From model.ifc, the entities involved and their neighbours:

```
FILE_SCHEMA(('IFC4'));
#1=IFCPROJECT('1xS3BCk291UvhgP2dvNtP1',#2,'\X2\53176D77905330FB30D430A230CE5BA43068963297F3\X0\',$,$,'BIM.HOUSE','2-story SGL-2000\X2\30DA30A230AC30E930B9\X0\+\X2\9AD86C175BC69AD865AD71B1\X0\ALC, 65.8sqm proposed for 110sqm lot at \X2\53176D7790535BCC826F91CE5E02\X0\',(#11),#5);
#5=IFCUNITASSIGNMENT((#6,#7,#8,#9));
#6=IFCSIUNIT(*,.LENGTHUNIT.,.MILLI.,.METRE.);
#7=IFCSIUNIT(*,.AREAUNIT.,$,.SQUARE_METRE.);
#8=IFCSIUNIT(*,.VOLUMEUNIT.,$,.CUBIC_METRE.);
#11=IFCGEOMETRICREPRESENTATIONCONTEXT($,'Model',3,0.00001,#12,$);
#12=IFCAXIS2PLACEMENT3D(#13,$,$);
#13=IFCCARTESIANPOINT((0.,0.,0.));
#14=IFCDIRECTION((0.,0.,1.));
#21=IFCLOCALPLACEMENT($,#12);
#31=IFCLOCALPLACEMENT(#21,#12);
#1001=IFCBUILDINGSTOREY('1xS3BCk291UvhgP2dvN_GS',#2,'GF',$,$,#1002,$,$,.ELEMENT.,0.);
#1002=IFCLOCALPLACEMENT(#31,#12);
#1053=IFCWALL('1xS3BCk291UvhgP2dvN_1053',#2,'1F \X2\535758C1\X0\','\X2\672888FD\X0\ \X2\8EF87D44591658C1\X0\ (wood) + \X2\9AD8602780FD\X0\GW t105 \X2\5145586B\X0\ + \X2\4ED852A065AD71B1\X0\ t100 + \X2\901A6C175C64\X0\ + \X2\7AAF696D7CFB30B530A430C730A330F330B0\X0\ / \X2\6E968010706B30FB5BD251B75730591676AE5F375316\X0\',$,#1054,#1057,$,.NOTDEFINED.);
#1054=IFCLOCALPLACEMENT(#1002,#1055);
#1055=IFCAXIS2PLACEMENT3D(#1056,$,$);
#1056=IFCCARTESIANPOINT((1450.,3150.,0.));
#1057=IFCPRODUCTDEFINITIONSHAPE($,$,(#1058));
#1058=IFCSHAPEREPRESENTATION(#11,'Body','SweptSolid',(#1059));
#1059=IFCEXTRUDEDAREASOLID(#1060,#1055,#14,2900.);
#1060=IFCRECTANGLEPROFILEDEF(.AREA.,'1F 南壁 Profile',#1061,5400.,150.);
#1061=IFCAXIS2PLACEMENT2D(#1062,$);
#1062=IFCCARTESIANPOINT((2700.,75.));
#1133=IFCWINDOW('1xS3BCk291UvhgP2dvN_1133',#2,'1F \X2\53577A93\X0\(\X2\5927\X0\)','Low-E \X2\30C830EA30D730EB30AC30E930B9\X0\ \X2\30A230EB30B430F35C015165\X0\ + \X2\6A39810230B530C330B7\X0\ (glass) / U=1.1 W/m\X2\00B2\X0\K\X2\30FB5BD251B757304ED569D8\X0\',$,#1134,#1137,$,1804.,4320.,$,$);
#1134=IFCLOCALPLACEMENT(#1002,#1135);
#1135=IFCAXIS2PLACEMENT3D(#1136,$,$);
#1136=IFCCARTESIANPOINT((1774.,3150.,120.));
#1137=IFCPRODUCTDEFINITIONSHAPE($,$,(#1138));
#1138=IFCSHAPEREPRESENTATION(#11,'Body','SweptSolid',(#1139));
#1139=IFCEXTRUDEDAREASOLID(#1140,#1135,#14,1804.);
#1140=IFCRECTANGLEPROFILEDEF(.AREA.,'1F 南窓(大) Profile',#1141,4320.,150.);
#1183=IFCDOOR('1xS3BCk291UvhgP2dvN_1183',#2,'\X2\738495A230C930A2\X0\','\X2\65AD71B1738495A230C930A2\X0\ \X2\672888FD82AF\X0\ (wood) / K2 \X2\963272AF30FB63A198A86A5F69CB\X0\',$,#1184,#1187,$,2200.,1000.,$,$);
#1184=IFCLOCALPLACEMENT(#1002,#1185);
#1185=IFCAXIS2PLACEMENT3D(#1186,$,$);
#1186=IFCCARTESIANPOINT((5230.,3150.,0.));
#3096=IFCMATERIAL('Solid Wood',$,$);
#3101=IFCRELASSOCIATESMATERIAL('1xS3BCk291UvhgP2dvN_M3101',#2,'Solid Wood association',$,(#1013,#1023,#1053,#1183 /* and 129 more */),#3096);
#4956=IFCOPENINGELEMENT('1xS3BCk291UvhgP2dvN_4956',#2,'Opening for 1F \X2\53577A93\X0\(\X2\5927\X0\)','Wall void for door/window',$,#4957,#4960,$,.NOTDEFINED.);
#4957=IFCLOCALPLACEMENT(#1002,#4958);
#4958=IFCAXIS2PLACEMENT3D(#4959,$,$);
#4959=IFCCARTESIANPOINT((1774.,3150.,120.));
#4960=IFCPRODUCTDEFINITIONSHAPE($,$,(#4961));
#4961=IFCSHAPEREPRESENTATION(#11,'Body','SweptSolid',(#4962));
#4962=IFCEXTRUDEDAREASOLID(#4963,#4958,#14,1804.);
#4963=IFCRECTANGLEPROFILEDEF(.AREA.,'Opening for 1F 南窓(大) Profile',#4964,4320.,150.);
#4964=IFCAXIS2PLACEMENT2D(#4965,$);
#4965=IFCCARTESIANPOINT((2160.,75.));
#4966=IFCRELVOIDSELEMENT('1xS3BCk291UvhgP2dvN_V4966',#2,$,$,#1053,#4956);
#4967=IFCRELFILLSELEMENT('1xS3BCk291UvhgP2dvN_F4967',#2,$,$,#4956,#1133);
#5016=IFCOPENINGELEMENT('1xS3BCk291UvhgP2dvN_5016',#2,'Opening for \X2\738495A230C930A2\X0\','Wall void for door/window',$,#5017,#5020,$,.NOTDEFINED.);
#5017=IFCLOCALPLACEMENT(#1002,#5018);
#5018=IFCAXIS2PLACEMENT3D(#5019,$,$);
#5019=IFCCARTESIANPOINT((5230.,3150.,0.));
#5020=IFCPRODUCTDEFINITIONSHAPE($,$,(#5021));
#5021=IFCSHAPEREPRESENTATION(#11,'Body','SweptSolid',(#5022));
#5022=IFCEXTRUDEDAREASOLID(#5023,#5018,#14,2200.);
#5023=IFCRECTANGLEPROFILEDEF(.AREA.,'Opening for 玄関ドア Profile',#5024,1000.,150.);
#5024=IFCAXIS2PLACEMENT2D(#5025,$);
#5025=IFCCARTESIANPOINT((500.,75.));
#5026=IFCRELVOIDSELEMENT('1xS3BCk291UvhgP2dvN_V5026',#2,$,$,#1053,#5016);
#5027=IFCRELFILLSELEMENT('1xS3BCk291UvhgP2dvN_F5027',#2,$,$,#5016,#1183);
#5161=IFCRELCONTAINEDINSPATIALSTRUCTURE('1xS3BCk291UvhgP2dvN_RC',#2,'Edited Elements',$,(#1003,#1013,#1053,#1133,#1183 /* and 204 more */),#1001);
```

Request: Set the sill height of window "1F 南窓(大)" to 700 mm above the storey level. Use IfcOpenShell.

```python
import numpy as np
import ifcopenshell
import ifcopenshell.api.geometry
import ifcopenshell.geom
import ifcopenshell.util.element
import ifcopenshell.util.placement
import ifcopenshell.util.shape
import ifcopenshell.util.unit

model = ifcopenshell.open("model.ifc")
unit_scale = ifcopenshell.util.unit.calculate_unit_scale(model)

window = model.by_guid("1xS3BCk291UvhgP2dvN_1133")
opening = window.FillsVoids[0].RelatingOpeningElement
storey = ifcopenshell.util.element.get_container(window, ifc_class="IfcBuildingStorey")
level = ifcopenshell.util.placement.get_local_placement(storey.ObjectPlacement)[2, 3]

# The opening's origin need not be at the sill, so measure its lowest point.
shape = ifcopenshell.geom.create_shape(ifcopenshell.geom.settings(), opening)
bottom = ifcopenshell.util.shape.get_shape_bottom_elevation(shape, shape.geometry) / unit_scale
dz = level + 700.0 - bottom

shift = np.array([0.0, 0.0, dz])
# The window is not placed relative to its opening, so move both.
for product in (opening, window):
    matrix = ifcopenshell.util.placement.get_local_placement(product.ObjectPlacement)
    matrix[:3, 3] += shift
    ifcopenshell.api.geometry.edit_object_placement(model, product=product, matrix=matrix, is_si=False)

print(f"moved by {dz * unit_scale:+.3f} m")

model.write("model_rev.ifc")
```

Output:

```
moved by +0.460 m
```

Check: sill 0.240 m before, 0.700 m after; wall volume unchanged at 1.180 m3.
